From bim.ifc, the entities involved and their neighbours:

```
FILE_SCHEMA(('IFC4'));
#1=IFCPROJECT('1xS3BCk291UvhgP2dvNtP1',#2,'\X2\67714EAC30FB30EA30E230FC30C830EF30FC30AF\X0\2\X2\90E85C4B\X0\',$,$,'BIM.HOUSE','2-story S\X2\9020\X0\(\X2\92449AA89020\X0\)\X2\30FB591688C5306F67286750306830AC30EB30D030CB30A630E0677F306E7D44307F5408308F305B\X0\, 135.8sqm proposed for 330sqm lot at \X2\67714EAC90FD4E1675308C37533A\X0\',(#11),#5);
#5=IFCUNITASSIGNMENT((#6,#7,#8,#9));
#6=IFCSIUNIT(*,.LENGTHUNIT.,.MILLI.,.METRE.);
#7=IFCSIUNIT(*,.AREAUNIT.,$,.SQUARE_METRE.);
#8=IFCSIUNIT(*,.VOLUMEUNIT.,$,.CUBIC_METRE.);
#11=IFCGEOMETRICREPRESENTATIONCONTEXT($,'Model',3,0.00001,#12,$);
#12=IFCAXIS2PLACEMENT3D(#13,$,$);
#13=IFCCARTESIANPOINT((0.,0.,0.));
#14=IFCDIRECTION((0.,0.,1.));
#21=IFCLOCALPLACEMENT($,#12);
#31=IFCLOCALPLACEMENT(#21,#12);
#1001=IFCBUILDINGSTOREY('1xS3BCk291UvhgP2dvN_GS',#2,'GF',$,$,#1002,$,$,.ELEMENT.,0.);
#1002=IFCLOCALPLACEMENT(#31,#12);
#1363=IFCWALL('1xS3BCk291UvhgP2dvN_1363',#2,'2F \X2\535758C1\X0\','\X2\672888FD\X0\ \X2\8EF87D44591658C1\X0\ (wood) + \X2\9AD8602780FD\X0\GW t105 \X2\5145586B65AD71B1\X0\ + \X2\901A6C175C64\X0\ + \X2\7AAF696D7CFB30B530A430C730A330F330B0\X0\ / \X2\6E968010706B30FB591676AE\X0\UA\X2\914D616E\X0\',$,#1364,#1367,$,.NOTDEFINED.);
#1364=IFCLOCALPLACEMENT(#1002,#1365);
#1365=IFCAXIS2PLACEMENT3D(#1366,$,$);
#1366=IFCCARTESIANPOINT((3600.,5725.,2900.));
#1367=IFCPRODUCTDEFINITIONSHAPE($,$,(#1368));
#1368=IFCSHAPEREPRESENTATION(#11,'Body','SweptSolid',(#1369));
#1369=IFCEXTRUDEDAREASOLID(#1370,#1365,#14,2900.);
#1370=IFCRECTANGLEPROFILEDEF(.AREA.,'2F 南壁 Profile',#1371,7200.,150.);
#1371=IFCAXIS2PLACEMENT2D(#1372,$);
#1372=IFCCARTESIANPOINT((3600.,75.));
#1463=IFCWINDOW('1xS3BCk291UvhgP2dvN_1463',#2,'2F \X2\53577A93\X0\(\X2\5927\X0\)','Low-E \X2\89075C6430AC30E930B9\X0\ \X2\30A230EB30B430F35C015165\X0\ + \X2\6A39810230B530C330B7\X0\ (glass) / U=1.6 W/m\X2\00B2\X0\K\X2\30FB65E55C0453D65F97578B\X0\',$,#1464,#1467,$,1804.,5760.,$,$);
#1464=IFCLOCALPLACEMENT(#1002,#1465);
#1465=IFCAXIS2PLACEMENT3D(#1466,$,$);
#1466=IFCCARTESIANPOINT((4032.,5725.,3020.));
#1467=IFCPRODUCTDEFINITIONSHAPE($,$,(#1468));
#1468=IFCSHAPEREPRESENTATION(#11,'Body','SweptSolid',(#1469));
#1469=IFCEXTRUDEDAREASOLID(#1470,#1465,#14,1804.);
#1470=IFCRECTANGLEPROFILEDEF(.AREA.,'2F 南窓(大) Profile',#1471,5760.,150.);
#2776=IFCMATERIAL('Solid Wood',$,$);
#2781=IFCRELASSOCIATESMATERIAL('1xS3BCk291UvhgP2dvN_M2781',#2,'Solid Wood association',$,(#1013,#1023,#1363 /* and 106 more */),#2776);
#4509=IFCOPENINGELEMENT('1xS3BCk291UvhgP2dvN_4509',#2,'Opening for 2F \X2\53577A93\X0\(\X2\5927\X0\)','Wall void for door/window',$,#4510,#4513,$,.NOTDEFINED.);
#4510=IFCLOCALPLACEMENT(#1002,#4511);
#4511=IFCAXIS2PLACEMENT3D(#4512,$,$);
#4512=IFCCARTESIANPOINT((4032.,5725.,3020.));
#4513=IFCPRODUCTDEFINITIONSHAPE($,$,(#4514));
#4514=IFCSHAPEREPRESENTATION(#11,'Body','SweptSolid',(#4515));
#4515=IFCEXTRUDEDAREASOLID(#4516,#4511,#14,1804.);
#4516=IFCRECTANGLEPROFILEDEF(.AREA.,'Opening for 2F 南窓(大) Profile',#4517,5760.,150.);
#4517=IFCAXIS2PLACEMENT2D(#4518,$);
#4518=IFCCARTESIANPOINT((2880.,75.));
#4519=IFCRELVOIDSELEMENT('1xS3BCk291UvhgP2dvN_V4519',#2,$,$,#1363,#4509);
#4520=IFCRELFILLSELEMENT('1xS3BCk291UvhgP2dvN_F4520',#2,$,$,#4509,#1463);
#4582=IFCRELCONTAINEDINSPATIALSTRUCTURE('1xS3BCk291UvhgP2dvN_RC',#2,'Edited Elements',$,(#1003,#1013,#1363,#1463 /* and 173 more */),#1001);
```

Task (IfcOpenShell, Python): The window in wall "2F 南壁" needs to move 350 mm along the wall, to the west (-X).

```python
import ifcopenshell
import ifcopenshell.api.geometry
import ifcopenshell.util.placement

model = ifcopenshell.open("bim.ifc")

window = model.by_guid("1xS3BCk291UvhgP2dvN_1463")
opening = window.FillsVoids[0].RelatingOpeningElement
wall = opening.VoidsElements[0].RelatingBuildingElement

wall_matrix = ifcopenshell.util.placement.get_local_placement(wall.ObjectPlacement)
shift = wall_matrix[:3, 0] * -350.0
before = ifcopenshell.util.placement.get_local_placement(window.ObjectPlacement)[:3, 3].copy()

# The window is not placed relative to its opening, so move both.
for product in (opening, window):
    matrix = ifcopenshell.util.placement.get_local_placement(product.ObjectPlacement)
    matrix[:3, 3] += shift
    ifcopenshell.api.geometry.edit_object_placement(model, product=product, matrix=matrix, is_si=False)

after = ifcopenshell.util.placement.get_local_placement(window.ObjectPlacement)[:3, 3]
print("window moved by", (after - before).round(3) + 0.0)

model.write("bim_rev.ifc")
```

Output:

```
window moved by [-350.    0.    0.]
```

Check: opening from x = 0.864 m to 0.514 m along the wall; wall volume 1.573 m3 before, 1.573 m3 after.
